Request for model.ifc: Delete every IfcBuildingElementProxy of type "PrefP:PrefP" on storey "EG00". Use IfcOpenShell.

First a look at what the model holds.

```python
import ifcopenshell
import ifcopenshell.util.element

model = ifcopenshell.open("model.ifc")
print(model.schema)
storey = next(s for s in model.by_type("IfcBuildingStorey") if s.Name == "EG00")
proxies = [e for e in ifcopenshell.util.element.get_decomposition(storey) if e.is_a("IfcBuildingElementProxy")]
seen = {}
for e in proxies:
    element_type = ifcopenshell.util.element.get_type(e)
    name = element_type.Name if element_type not in (None, e) else None
    seen[name] = seen.get(name, 0) + 1
for name, count in sorted(seen.items(), key=str):
    print(count, "x", name)
```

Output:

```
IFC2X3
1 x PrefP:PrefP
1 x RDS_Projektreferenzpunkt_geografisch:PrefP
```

```python
import ifcopenshell
import ifcopenshell.api.root
import ifcopenshell.util.element

model = ifcopenshell.open("model.ifc")

storey = next(s for s in model.by_type("IfcBuildingStorey") if s.Name == "EG00")
proxies = [e for e in ifcopenshell.util.element.get_decomposition(storey) if e.is_a("IfcBuildingElementProxy")]
targets = [e for e in proxies if (t := ifcopenshell.util.element.get_type(e)) not in (None, e) and t.Name == "PrefP:PrefP"]

for e in targets:
    ifcopenshell.api.root.remove_product(model, product=e)
print(len(targets), "removed")

model.write("model_rev.ifc")
```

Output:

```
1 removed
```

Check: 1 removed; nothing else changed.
